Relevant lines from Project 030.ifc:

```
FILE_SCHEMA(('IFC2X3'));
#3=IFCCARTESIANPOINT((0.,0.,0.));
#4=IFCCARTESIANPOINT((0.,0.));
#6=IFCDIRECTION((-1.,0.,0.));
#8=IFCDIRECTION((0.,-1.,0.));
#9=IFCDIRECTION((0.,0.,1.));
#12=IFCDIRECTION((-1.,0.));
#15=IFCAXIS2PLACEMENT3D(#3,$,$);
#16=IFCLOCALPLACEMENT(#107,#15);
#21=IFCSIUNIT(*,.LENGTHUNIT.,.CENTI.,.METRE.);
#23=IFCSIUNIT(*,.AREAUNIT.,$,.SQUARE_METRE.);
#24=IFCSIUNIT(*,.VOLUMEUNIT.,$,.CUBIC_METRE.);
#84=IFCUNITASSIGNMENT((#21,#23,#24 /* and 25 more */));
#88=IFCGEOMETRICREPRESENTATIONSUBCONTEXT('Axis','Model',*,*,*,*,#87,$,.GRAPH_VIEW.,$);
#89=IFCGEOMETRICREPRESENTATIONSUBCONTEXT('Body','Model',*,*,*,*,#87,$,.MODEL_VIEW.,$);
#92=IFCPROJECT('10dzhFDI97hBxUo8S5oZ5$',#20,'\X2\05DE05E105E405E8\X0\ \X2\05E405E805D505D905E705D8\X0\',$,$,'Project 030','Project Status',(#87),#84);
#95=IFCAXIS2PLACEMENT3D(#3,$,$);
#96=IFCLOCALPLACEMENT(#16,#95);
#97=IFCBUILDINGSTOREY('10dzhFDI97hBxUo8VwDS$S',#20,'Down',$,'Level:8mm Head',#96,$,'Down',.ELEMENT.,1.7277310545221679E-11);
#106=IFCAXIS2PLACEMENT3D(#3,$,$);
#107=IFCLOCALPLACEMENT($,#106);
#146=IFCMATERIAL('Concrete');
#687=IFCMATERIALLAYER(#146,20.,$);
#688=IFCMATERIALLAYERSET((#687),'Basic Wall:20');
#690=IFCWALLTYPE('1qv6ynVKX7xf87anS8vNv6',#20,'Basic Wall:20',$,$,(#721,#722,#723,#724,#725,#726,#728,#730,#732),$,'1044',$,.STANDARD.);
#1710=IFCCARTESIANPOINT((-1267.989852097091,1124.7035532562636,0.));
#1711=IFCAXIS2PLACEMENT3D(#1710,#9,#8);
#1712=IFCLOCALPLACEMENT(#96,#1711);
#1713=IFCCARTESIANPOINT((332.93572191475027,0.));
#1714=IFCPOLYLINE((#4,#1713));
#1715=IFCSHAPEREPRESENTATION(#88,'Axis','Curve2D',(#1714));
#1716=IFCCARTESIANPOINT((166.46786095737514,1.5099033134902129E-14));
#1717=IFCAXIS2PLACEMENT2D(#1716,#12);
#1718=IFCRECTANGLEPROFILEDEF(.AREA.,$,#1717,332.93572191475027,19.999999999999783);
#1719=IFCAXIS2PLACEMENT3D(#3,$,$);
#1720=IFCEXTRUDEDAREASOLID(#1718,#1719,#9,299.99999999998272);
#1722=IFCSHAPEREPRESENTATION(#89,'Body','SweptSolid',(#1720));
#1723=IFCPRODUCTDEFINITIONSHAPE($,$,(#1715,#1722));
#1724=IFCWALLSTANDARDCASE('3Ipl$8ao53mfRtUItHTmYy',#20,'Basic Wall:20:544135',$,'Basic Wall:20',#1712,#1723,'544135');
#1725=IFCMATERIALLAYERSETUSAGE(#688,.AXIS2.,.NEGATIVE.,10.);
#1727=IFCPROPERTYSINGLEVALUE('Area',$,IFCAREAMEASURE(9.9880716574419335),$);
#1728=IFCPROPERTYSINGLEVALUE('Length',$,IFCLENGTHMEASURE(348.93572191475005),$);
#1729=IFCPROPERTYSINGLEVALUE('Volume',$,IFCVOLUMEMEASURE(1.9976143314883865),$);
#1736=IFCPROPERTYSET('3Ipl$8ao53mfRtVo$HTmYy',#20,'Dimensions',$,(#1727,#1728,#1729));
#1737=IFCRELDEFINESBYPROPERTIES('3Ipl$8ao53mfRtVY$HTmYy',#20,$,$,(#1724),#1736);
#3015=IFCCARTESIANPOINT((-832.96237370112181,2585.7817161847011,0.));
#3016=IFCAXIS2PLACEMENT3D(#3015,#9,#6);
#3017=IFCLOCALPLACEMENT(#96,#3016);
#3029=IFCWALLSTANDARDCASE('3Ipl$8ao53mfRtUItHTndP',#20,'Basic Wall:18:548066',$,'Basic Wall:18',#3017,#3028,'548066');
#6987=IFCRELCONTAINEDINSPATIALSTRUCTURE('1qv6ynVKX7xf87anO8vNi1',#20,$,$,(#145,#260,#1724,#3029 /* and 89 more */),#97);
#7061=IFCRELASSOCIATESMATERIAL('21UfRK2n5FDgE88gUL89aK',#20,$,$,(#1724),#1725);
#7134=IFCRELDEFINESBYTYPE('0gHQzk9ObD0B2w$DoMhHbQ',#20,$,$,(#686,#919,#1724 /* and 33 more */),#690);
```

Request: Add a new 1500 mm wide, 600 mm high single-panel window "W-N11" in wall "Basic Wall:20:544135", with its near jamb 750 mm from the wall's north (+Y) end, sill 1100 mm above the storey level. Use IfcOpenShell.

```python
import numpy as np
import ifcopenshell
import ifcopenshell.api.feature
import ifcopenshell.api.geometry
import ifcopenshell.api.pset
import ifcopenshell.api.root
import ifcopenshell.api.spatial
import ifcopenshell.api.type
import ifcopenshell.geom
import ifcopenshell.util.element
import ifcopenshell.util.placement
import ifcopenshell.util.representation
import ifcopenshell.util.shape
import ifcopenshell.util.unit

model = ifcopenshell.open("Project 030.ifc")
unit_scale = ifcopenshell.util.unit.calculate_unit_scale(model)
area_scale = ifcopenshell.util.unit.calculate_unit_scale(model, "AREAUNIT")
volume_scale = ifcopenshell.util.unit.calculate_unit_scale(model, "VOLUMEUNIT")
settings = ifcopenshell.geom.settings()


def volume(element):
    """Net volume in cubic metres, openings subtracted."""
    shape = ifcopenshell.geom.create_shape(settings, element)
    return ifcopenshell.util.shape.get_volume(shape.geometry)


wall = model.by_id(1724)
storey = ifcopenshell.util.element.get_container(wall, ifc_class="IfcBuildingStorey")
context = ifcopenshell.util.representation.get_context(model, "Model", "Body", "MODEL_VIEW")
before = volume(wall)

width, height, from_end, sill = 1.5, 0.6, 0.75, 1.1  # metres

# The wall runs along its own X axis, and the end named is its -X end.
wall_shape = ifcopenshell.geom.create_shape(settings, wall)
x, y, z = ifcopenshell.util.shape.get_vertices(wall_shape.geometry).T
start = x.min() + from_end
face, thickness = float(y.min()), float(y.max() - y.min())
wall_matrix = ifcopenshell.util.placement.get_local_placement(wall.ObjectPlacement)
level = ifcopenshell.util.placement.get_local_placement(storey.ObjectPlacement)[2, 3]


def in_wall(x, y):
    """Placement at x, y metres in the wall's axes, at sill height."""
    matrix = wall_matrix.copy()
    matrix[:, 3] = wall_matrix @ np.array([x / unit_scale, y / unit_scale, 0.0, 1.0])
    matrix[2, 3] = level + sill / unit_scale
    return matrix


# Opening: a box that overshoots both wall faces by 50 mm.
opening = ifcopenshell.api.root.create_entity(model, ifc_class="IfcOpeningElement")
box = ifcopenshell.api.geometry.add_wall_representation(
    model, context=context, length=width, height=height, thickness=thickness + 0.1
)
ifcopenshell.api.geometry.assign_representation(model, product=opening, representation=box)
ifcopenshell.api.geometry.edit_object_placement(model, product=opening, matrix=in_wall(start, face - 0.05), is_si=False)
ifcopenshell.api.feature.add_feature(model, feature=opening, element=wall)

window = ifcopenshell.api.root.create_entity(model, ifc_class="IfcWindow", name="W-N11")
window.OverallWidth, window.OverallHeight = width / unit_scale, height / unit_scale
body = ifcopenshell.api.geometry.add_window_representation(
    model,
    context=context,
    overall_width=window.OverallWidth,
    overall_height=window.OverallHeight,
    partition_type="SINGLE_PANEL",
)
ifcopenshell.api.geometry.assign_representation(model, product=window, representation=body)
ifcopenshell.api.spatial.assign_container(model, products=[window], relating_structure=storey)
fills = ifcopenshell.api.feature.add_filling(model, opening=opening, element=window)
fills.OwnerHistory = window.OwnerHistory  # required in IFC2X3

# IFC2X3 keeps the operation on the window style.
style = ifcopenshell.api.root.create_entity(model, ifc_class="IfcWindowStyle", name="W-N11")
style.OperationType, style.ConstructionType = "SINGLE_PANEL", "NOTDEFINED"
style.ParameterTakesPrecedence = style.Sizeable = False
ifcopenshell.api.type.assign_type(model, related_objects=[window], relating_type=style)

# Centre the window in the wall's thickness.
ifcopenshell.api.geometry.edit_object_placement(model, product=window, matrix=in_wall(start, face), is_si=False)
window_shape = ifcopenshell.geom.create_shape(settings, window)
depth = ifcopenshell.util.shape.get_vertices(window_shape.geometry)[:, 1]
offset = face + thickness / 2 - (depth.min() + depth.max()) / 2
ifcopenshell.api.geometry.edit_object_placement(model, product=window, matrix=in_wall(start, offset), is_si=False)

after = volume(wall)

# Update the wall's stored quantities.
pset = model.by_id(ifcopenshell.util.element.get_pset(wall, "Dimensions", should_inherit=False)["id"])
ifcopenshell.api.pset.edit_pset(model, pset=pset, properties={
    "Area": model.create_entity("IfcAreaMeasure", after / thickness / area_scale),
    "Volume": model.create_entity("IfcVolumeMeasure", after / volume_scale),
})

print(f"wall volume {before:.3f} -> {after:.3f} m3")

model.write("Project 030-out.ifc")
```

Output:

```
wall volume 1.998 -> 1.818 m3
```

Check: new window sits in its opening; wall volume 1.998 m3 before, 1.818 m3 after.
